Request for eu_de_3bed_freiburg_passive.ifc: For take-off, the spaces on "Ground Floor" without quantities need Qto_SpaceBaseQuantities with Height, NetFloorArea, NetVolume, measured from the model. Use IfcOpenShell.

First a look at what the model holds.

```python
import ifcopenshell
import ifcopenshell.util.element
import ifcopenshell.util.unit

model = ifcopenshell.open("eu_de_3bed_freiburg_passive.ifc")
print(model.schema)
for unit_type in ("LENGTHUNIT", "AREAUNIT", "VOLUMEUNIT"):
    print(unit_type, ifcopenshell.util.unit.calculate_unit_scale(model, unit_type))
storey = next(s for s in model.by_type("IfcBuildingStorey") if s.Name == "Ground Floor")
spaces = [e for e in ifcopenshell.util.element.get_decomposition(storey) if e.is_a("IfcSpace")]
for e in sorted(spaces, key=lambda e: e.id()):
    print(e.id(), e.is_a(), e.Name, list(ifcopenshell.util.element.get_psets(e, qtos_only=True)), sep=" | ")
```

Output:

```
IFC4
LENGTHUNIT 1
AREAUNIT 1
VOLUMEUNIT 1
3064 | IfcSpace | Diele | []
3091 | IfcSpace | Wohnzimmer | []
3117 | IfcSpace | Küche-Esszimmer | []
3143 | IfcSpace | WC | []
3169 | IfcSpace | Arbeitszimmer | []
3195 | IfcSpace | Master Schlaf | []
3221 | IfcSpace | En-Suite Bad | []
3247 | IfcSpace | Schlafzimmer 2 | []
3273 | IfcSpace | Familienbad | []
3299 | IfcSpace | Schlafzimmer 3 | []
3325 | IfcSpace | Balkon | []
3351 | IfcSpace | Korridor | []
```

```python
import ifcopenshell
import ifcopenshell.api.pset
import ifcopenshell.geom
import ifcopenshell.util.element
import ifcopenshell.util.shape
import ifcopenshell.util.unit

model = ifcopenshell.open("eu_de_3bed_freiburg_passive.ifc")
unit_scale = ifcopenshell.util.unit.calculate_unit_scale(model)
area_scale = ifcopenshell.util.unit.calculate_unit_scale(model, "AREAUNIT")
volume_scale = ifcopenshell.util.unit.calculate_unit_scale(model, "VOLUMEUNIT")
settings = ifcopenshell.geom.settings()

storey = next(s for s in model.by_type("IfcBuildingStorey") if s.Name == "Ground Floor")
spaces = [e for e in ifcopenshell.util.element.get_decomposition(storey) if e.is_a("IfcSpace")]

for e in sorted(spaces, key=lambda e: e.id()):
    if ifcopenshell.util.element.get_psets(e, qtos_only=True, should_inherit=False):
        continue
    # Geometry comes back in metres, in the element's own axes.
    shape = ifcopenshell.geom.create_shape(settings, e)
    values = {
        "Height": ifcopenshell.util.shape.get_z(shape.geometry) / unit_scale,
        "NetFloorArea": ifcopenshell.util.shape.get_footprint_area(shape.geometry) / area_scale,
        "NetVolume": ifcopenshell.util.shape.get_volume(shape.geometry) / volume_scale,
    }
    qto = ifcopenshell.api.pset.add_qto(model, product=e, name="Qto_SpaceBaseQuantities")
    ifcopenshell.api.pset.edit_qto(model, qto=qto, properties=values)
    print(e.id(), {k: round(v, 3) for k, v in values.items()})

model.write("eu_de_3bed_freiburg_passive-out.ifc")
```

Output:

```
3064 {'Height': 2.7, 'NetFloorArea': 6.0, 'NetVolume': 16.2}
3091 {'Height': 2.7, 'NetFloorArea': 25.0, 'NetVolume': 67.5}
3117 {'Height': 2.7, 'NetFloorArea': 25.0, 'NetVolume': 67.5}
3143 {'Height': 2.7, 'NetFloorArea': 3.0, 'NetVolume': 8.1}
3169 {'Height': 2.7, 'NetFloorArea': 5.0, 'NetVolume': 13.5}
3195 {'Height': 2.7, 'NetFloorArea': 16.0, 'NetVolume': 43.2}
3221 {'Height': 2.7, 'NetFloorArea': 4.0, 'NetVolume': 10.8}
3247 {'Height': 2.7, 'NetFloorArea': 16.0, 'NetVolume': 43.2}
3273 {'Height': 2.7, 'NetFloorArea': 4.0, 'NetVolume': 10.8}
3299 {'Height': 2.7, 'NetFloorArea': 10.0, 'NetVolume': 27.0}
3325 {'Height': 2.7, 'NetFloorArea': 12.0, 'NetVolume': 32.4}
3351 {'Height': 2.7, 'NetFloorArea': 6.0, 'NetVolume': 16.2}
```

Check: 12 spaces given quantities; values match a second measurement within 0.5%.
